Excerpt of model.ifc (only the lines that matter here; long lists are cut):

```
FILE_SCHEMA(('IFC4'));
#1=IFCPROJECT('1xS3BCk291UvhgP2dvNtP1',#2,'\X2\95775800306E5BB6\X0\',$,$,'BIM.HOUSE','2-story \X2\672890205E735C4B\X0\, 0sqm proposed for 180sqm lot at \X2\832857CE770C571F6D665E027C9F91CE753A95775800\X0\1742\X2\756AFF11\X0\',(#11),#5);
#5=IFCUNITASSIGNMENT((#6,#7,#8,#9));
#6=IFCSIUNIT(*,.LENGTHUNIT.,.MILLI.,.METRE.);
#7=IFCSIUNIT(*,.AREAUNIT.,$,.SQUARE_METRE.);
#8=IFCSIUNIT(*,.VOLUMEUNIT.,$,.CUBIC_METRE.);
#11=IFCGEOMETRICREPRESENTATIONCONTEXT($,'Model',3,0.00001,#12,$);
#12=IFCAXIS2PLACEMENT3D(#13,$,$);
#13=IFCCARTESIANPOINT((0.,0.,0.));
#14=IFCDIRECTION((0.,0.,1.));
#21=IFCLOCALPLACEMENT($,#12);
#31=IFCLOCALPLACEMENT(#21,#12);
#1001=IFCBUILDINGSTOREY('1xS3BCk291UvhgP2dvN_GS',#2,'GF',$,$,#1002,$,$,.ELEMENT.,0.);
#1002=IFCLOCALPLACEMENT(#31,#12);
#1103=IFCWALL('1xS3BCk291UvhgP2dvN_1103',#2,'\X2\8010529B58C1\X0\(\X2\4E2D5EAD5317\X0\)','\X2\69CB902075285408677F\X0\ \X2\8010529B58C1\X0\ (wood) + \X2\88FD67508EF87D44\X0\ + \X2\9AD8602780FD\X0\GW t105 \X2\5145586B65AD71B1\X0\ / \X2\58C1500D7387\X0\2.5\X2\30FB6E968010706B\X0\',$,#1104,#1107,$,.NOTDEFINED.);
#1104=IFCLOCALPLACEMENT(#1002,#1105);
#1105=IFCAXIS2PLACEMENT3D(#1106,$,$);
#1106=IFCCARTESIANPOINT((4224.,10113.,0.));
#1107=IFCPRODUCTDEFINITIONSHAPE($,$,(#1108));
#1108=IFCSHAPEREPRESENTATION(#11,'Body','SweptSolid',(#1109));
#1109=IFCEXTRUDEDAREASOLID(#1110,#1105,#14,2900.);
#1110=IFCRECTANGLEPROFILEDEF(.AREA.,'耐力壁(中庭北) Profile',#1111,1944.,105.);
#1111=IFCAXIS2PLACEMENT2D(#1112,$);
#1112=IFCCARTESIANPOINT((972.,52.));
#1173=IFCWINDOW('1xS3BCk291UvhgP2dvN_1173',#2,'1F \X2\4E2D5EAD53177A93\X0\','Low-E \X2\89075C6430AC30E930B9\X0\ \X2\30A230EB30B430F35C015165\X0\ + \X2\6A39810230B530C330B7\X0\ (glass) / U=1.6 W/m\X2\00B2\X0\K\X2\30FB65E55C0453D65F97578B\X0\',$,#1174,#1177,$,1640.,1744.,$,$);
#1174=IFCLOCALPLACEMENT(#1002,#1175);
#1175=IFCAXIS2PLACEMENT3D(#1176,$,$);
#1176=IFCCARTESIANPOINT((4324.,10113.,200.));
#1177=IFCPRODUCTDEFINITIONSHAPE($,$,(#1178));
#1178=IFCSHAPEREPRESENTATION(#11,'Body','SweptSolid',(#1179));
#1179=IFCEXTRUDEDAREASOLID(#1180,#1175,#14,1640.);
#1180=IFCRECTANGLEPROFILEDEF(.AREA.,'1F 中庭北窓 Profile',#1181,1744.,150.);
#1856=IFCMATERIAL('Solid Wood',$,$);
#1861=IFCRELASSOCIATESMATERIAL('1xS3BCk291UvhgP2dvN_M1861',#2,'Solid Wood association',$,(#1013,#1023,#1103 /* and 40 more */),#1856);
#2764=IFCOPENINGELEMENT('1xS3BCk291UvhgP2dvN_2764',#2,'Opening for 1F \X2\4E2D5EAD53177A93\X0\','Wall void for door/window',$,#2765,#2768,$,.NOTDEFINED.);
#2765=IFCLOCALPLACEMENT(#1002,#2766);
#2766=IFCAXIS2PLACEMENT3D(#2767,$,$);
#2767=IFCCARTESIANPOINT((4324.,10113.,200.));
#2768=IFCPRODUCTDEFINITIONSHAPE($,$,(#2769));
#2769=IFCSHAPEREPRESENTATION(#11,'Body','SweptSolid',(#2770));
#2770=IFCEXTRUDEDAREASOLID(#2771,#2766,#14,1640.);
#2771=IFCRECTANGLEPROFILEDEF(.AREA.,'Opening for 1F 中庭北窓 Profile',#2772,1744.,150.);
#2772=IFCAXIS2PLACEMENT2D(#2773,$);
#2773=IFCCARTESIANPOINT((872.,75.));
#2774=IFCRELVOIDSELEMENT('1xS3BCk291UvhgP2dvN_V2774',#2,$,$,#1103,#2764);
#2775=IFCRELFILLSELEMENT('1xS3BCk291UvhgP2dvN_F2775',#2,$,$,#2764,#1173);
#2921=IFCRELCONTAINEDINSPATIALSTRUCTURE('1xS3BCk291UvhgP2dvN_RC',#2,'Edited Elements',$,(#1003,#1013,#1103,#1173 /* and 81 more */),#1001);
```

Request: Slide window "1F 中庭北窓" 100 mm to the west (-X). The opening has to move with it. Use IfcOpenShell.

```python
import ifcopenshell
import ifcopenshell.api.geometry
import ifcopenshell.util.placement
import ifcopenshell.util.unit

model = ifcopenshell.open("model.ifc")
unit_scale = ifcopenshell.util.unit.calculate_unit_scale(model)

window = model.by_id(1173)
opening = window.FillsVoids[0].RelatingOpeningElement
wall = opening.VoidsElements[0].RelatingBuildingElement

wall_matrix = ifcopenshell.util.placement.get_local_placement(wall.ObjectPlacement)
shift = wall_matrix[:3, 0] * -0.1 / unit_scale
before = ifcopenshell.util.placement.get_local_placement(window.ObjectPlacement)[:3, 3].copy()

# The window is not placed relative to its opening, so move both.
for product in (opening, window):
    matrix = ifcopenshell.util.placement.get_local_placement(product.ObjectPlacement)
    matrix[:3, 3] += shift
    ifcopenshell.api.geometry.edit_object_placement(model, product=product, matrix=matrix, is_si=False)

after = ifcopenshell.util.placement.get_local_placement(window.ObjectPlacement)[:3, 3]
print("window moved by", (after - before).round(3) + 0.0)

model.write("model_rev.ifc")
```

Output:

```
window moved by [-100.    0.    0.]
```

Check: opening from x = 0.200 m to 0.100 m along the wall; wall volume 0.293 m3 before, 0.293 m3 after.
